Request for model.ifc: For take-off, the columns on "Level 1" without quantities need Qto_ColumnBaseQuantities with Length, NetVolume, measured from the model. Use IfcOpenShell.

First a look at what the model holds.

```python
import ifcopenshell
import ifcopenshell.util.element
import ifcopenshell.util.unit

model = ifcopenshell.open("model.ifc")
print(model.schema)
for unit_type in ("LENGTHUNIT", "AREAUNIT", "VOLUMEUNIT"):
    print(unit_type, ifcopenshell.util.unit.calculate_unit_scale(model, unit_type))
storey = next(s for s in model.by_type("IfcBuildingStorey") if s.Name == "Level 1")
columns = [e for e in ifcopenshell.util.element.get_decomposition(storey) if e.is_a("IfcColumn")]
for e in sorted(columns, key=lambda e: e.id()):
    print(e.id(), e.is_a(), e.Name, list(ifcopenshell.util.element.get_psets(e, qtos_only=True)), sep=" | ")
```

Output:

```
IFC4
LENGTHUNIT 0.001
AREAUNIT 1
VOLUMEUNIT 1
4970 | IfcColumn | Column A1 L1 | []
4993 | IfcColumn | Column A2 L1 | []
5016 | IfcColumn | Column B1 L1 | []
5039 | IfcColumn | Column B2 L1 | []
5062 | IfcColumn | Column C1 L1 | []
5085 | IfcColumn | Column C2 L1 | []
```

```python
import ifcopenshell
import ifcopenshell.api.pset
import ifcopenshell.geom
import ifcopenshell.util.element
import ifcopenshell.util.shape
import ifcopenshell.util.unit

model = ifcopenshell.open("model.ifc")
unit_scale = ifcopenshell.util.unit.calculate_unit_scale(model)
volume_scale = ifcopenshell.util.unit.calculate_unit_scale(model, "VOLUMEUNIT")
settings = ifcopenshell.geom.settings()

storey = next(s for s in model.by_type("IfcBuildingStorey") if s.Name == "Level 1")
columns = [e for e in ifcopenshell.util.element.get_decomposition(storey) if e.is_a("IfcColumn")]

for e in sorted(columns, key=lambda e: e.id()):
    if ifcopenshell.util.element.get_psets(e, qtos_only=True, should_inherit=False):
        continue
    # Geometry comes back in metres, in the element's own axes.
    shape = ifcopenshell.geom.create_shape(settings, e)
    values = {
        "Length": ifcopenshell.util.shape.get_z(shape.geometry) / unit_scale,
        "NetVolume": ifcopenshell.util.shape.get_volume(shape.geometry) / volume_scale,
    }
    qto = ifcopenshell.api.pset.add_qto(model, product=e, name="Qto_ColumnBaseQuantities")
    ifcopenshell.api.pset.edit_qto(model, qto=qto, properties=values)
    print(e.id(), {k: round(v, 3) for k, v in values.items()})

model.write("model-out.ifc")
```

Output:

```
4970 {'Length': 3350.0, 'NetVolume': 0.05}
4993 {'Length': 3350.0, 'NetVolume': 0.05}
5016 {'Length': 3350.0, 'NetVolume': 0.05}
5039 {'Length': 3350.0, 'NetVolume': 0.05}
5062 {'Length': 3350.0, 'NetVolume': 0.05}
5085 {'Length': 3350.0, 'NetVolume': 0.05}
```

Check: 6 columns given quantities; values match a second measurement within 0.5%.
